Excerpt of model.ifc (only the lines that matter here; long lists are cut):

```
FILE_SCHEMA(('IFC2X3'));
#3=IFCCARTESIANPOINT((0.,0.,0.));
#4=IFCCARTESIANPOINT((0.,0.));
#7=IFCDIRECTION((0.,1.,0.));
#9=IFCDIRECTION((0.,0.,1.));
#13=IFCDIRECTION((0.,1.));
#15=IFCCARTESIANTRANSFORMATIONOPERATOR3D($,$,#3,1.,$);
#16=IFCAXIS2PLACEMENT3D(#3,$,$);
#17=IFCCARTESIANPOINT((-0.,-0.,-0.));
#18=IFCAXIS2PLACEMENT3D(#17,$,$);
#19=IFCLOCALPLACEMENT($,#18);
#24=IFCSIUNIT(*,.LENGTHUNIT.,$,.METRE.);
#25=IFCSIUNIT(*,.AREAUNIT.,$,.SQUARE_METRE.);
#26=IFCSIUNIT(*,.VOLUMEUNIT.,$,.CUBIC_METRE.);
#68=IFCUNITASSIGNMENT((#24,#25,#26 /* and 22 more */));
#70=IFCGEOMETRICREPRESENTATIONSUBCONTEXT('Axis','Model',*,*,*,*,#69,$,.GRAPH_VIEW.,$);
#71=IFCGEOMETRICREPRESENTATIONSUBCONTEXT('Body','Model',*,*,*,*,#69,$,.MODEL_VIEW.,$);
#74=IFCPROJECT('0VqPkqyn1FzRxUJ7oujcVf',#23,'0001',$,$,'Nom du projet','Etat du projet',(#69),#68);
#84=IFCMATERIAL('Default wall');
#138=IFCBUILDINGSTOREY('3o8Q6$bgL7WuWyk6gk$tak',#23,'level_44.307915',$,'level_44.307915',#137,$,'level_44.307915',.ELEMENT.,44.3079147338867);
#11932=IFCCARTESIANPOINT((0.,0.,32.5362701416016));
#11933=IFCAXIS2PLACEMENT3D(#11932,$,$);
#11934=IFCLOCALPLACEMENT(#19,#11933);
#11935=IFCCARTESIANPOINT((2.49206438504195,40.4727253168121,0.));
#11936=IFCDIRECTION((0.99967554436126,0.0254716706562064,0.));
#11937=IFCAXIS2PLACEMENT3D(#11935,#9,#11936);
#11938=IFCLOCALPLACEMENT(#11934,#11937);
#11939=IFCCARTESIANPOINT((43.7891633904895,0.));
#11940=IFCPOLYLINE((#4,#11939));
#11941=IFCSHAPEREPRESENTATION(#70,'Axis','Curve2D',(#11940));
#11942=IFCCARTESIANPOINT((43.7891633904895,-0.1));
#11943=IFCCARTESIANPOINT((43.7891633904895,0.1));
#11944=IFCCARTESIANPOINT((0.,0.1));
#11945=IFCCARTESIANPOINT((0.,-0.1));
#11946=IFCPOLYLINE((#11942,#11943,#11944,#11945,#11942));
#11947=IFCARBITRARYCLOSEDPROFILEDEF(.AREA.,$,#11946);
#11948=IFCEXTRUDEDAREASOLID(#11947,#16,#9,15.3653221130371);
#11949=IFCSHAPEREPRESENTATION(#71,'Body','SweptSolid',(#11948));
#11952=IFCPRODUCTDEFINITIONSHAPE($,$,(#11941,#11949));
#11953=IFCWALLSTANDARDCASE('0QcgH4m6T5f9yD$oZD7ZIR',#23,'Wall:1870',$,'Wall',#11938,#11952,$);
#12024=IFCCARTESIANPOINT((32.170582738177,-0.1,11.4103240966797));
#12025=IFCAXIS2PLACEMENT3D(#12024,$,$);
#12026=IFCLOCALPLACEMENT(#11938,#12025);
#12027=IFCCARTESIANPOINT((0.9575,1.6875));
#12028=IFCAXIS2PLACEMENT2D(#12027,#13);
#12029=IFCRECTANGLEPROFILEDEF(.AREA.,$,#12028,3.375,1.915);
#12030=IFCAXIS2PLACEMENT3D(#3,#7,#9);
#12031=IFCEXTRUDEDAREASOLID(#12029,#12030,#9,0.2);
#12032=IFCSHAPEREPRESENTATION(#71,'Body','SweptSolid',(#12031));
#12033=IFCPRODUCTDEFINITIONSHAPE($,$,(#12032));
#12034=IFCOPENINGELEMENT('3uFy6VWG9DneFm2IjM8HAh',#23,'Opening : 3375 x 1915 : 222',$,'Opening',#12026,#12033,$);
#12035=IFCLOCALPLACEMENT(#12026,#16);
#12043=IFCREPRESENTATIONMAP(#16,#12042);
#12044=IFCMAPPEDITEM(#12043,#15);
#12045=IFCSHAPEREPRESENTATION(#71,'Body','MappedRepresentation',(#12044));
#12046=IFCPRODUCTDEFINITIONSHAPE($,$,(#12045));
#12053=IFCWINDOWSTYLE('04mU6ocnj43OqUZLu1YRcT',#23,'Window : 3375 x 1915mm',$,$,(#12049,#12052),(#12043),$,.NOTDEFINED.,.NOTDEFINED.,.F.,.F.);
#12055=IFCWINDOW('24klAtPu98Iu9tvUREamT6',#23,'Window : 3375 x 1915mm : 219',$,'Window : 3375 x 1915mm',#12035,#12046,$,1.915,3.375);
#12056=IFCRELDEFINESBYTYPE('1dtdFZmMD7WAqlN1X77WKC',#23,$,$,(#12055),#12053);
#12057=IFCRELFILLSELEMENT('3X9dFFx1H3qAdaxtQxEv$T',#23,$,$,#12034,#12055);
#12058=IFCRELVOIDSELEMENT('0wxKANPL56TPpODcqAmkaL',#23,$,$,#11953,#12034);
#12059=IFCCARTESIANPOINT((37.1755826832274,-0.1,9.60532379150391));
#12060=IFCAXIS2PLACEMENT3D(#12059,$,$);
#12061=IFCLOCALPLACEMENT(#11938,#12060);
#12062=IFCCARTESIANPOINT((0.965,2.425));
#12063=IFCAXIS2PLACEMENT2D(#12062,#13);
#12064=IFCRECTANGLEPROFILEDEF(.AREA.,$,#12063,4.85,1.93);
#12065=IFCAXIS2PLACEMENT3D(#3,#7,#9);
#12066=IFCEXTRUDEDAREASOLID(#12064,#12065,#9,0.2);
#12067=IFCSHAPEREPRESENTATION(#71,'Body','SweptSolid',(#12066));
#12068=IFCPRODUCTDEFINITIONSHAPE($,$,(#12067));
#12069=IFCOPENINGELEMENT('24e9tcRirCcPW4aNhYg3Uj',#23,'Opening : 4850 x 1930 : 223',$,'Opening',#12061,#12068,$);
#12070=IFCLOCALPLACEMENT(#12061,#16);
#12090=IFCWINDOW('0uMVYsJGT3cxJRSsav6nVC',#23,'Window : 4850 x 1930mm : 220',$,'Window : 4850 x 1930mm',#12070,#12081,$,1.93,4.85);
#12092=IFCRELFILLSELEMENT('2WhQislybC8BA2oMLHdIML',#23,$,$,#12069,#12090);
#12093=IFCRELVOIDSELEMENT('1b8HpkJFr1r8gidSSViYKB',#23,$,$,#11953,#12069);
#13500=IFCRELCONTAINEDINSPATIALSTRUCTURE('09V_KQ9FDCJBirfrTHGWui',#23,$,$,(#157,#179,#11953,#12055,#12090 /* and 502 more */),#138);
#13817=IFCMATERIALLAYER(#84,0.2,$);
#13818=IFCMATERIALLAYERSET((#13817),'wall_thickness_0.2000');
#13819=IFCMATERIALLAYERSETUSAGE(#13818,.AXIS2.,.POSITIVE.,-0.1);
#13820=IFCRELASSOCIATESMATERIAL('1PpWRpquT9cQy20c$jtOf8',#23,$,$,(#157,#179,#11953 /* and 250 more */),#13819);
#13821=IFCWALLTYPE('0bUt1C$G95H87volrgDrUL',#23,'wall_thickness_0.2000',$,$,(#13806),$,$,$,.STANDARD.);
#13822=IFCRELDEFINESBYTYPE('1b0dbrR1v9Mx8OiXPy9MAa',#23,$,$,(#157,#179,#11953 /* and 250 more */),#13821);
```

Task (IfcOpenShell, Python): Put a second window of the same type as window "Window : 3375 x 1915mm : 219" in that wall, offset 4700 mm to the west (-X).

```python
import ifcopenshell
import ifcopenshell.api.feature
import ifcopenshell.api.geometry
import ifcopenshell.api.root
import ifcopenshell.geom
import ifcopenshell.util.element
import ifcopenshell.util.placement
import ifcopenshell.util.shape
import ifcopenshell.util.unit

model = ifcopenshell.open("model.ifc")
unit_scale = ifcopenshell.util.unit.calculate_unit_scale(model)
settings = ifcopenshell.geom.settings()


def volume(element):
    """Net volume in cubic metres, openings subtracted."""
    shape = ifcopenshell.geom.create_shape(settings, element)
    return ifcopenshell.util.shape.get_volume(shape.geometry)


window = model.by_guid("24klAtPu98Iu9tvUREamT6")
opening = window.FillsVoids[0].RelatingOpeningElement
wall = opening.VoidsElements[0].RelatingBuildingElement
before = volume(wall)
shift = ifcopenshell.util.placement.get_local_placement(wall.ObjectPlacement)[:3, 0] * -4.7 / unit_scale

# copy_class copies the void relationship, type, container and properties, but no geometry.
new_opening = ifcopenshell.api.root.copy_class(model, product=opening)
new_opening.Representation = ifcopenshell.util.element.copy_deep(
    model, opening.Representation, exclude=["IfcGeometricRepresentationContext", "IfcRepresentationMap"]
)
new_opening.Name = "Opening : 3375 x 1915"
new_window = ifcopenshell.api.root.copy_class(model, product=window)
new_window.Representation = ifcopenshell.util.element.copy_deep(
    model, window.Representation, exclude=["IfcGeometricRepresentationContext", "IfcRepresentationMap"]
)
new_window.Name = "Window : 3375 x 1915mm"
fills = ifcopenshell.api.feature.add_filling(model, opening=new_opening, element=new_window)
fills.OwnerHistory = new_window.OwnerHistory  # required in IFC2X3

for old, new in ((opening, new_opening), (window, new_window)):
    matrix = ifcopenshell.util.placement.get_local_placement(old.ObjectPlacement)
    matrix[:3, 3] += shift
    ifcopenshell.api.geometry.edit_object_placement(model, product=new, matrix=matrix, is_si=False)

after = volume(wall)

print(f"wall volume {before:.3f} -> {after:.3f} m3")

model.write("model-out.ifc")
```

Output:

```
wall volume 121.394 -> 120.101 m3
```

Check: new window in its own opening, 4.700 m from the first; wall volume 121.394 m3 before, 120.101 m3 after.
